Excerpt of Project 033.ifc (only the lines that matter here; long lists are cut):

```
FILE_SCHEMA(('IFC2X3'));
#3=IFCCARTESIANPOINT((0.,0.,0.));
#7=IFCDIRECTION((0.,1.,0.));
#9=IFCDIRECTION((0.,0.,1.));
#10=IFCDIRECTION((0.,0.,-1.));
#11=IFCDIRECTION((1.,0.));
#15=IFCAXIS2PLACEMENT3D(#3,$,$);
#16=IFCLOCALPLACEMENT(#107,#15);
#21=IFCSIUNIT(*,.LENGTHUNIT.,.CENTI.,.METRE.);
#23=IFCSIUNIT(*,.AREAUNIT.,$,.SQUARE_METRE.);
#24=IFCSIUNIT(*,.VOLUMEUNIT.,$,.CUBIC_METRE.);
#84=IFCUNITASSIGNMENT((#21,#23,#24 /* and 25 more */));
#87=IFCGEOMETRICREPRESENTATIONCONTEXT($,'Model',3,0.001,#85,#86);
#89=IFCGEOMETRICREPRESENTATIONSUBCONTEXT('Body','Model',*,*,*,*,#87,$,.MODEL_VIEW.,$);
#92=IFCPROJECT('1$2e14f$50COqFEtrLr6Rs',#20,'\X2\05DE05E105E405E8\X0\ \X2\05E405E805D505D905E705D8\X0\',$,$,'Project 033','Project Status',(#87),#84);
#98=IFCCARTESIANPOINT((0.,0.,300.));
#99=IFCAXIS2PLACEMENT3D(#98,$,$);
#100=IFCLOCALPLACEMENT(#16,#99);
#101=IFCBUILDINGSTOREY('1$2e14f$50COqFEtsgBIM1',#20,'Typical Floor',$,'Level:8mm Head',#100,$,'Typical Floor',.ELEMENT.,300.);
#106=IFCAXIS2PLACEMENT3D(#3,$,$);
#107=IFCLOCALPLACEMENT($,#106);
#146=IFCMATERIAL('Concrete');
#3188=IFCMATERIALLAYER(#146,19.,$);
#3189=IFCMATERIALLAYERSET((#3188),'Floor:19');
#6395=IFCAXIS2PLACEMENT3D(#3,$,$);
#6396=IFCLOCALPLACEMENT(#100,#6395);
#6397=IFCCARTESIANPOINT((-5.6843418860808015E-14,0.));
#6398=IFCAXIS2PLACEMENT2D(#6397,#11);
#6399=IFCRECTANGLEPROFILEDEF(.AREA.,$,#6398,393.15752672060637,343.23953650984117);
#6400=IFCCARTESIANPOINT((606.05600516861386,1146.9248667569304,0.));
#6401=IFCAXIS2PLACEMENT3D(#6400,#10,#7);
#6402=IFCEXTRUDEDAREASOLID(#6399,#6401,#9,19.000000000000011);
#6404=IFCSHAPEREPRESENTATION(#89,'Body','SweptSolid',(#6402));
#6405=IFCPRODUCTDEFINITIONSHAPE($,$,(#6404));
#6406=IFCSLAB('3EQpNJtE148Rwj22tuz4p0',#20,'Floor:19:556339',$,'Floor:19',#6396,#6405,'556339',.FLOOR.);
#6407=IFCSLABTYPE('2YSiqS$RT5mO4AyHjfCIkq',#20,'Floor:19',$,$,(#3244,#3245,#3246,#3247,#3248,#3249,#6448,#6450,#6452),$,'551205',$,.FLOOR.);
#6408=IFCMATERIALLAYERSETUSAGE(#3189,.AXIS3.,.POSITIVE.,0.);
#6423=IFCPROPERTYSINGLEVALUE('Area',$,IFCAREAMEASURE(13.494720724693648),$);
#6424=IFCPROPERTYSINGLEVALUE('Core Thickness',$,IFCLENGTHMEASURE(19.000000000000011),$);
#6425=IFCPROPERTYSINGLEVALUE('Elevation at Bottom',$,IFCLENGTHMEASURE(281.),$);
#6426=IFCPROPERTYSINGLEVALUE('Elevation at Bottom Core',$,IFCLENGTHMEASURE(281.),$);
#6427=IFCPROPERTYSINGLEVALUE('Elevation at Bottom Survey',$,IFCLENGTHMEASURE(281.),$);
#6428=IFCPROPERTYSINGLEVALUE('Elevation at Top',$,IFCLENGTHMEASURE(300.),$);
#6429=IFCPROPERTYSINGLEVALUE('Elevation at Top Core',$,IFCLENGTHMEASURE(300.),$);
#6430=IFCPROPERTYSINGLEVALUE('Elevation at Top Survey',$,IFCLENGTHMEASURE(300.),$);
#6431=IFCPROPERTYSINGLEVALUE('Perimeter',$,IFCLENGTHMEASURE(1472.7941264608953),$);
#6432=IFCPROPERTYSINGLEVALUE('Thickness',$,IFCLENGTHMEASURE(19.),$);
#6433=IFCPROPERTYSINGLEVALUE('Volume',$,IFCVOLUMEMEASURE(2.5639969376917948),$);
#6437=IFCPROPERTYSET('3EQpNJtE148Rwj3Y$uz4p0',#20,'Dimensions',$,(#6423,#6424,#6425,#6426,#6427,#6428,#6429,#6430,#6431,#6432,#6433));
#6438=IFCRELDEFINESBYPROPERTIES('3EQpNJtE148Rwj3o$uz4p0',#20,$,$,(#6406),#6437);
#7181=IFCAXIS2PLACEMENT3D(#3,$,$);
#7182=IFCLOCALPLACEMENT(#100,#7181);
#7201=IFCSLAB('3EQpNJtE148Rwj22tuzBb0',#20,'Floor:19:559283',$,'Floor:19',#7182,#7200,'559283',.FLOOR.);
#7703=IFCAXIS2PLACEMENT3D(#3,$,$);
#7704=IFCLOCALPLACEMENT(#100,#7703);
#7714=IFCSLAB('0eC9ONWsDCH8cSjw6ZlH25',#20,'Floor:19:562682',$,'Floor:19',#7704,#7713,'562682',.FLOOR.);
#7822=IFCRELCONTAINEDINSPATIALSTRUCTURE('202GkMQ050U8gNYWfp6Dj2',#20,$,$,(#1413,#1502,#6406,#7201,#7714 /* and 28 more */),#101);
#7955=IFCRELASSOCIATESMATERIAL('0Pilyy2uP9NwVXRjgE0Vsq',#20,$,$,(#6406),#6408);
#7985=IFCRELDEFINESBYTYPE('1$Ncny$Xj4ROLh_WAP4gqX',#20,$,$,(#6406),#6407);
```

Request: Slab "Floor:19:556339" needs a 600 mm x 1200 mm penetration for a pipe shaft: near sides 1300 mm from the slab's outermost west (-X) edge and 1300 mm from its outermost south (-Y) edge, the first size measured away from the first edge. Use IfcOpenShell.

```python
import numpy as np
import ifcopenshell
import ifcopenshell.api.feature
import ifcopenshell.api.geometry
import ifcopenshell.api.pset
import ifcopenshell.api.root
import ifcopenshell.geom
import ifcopenshell.util.element
import ifcopenshell.util.placement
import ifcopenshell.util.representation
import ifcopenshell.util.shape
import ifcopenshell.util.unit

model = ifcopenshell.open("Project 033.ifc")
unit_scale = ifcopenshell.util.unit.calculate_unit_scale(model)
area_scale = ifcopenshell.util.unit.calculate_unit_scale(model, "AREAUNIT")
volume_scale = ifcopenshell.util.unit.calculate_unit_scale(model, "VOLUMEUNIT")
settings = ifcopenshell.geom.settings()


def volume(element):
    """Net volume in cubic metres, openings subtracted."""
    shape = ifcopenshell.geom.create_shape(settings, element)
    return ifcopenshell.util.shape.get_volume(shape.geometry)


slab = model.by_id(6406)
before = volume(slab)

# Extent in the slab's own axes, in metres. The edges named are its -X and -Y sides.
slab_shape = ifcopenshell.geom.create_shape(settings, slab)
vertices = ifcopenshell.util.shape.get_vertices(slab_shape.geometry)
x_min, y_min, bottom = vertices.min(axis=0)
top = vertices[:, 2].max()

opening = ifcopenshell.api.root.create_entity(model, ifc_class="IfcOpeningElement", name="Pipe shaft opening")
context = ifcopenshell.util.representation.get_context(model, "Model", "Body", "MODEL_VIEW")
width, depth = 0.6, 1.2
outline = [(0.0, 0.0), (width, 0.0), (width, depth), (0.0, depth), (0.0, 0.0)]
# Overshoot both faces by 50 mm so the cut is clean.
shape = ifcopenshell.api.geometry.add_slab_representation(
    model, context=context, depth=top - bottom + 0.1, polyline=outline
)
ifcopenshell.api.geometry.assign_representation(model, product=opening, representation=shape)

matrix = ifcopenshell.util.placement.get_local_placement(slab.ObjectPlacement)
matrix[:, 3] = matrix @ np.append(np.array([x_min + 1.3, y_min + 1.3, bottom - 0.05]) / unit_scale, 1.0)
ifcopenshell.api.geometry.edit_object_placement(model, product=opening, matrix=matrix, is_si=False)
ifcopenshell.api.feature.add_feature(model, feature=opening, element=slab)

after = volume(slab)

# Update the slab's stored quantities.
pset = model.by_id(ifcopenshell.util.element.get_pset(slab, "Dimensions", should_inherit=False)["id"])
ifcopenshell.api.pset.edit_pset(model, pset=pset, properties={
    "Area": model.create_entity("IfcAreaMeasure", after / (top - bottom) / area_scale),
    "Volume": model.create_entity("IfcVolumeMeasure", after / volume_scale),
})

print(f"slab volume {before:.3f} -> {after:.3f} m3")

model.write("Project 033_v2.ifc")
```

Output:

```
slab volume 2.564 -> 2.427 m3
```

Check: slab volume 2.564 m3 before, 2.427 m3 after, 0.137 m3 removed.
